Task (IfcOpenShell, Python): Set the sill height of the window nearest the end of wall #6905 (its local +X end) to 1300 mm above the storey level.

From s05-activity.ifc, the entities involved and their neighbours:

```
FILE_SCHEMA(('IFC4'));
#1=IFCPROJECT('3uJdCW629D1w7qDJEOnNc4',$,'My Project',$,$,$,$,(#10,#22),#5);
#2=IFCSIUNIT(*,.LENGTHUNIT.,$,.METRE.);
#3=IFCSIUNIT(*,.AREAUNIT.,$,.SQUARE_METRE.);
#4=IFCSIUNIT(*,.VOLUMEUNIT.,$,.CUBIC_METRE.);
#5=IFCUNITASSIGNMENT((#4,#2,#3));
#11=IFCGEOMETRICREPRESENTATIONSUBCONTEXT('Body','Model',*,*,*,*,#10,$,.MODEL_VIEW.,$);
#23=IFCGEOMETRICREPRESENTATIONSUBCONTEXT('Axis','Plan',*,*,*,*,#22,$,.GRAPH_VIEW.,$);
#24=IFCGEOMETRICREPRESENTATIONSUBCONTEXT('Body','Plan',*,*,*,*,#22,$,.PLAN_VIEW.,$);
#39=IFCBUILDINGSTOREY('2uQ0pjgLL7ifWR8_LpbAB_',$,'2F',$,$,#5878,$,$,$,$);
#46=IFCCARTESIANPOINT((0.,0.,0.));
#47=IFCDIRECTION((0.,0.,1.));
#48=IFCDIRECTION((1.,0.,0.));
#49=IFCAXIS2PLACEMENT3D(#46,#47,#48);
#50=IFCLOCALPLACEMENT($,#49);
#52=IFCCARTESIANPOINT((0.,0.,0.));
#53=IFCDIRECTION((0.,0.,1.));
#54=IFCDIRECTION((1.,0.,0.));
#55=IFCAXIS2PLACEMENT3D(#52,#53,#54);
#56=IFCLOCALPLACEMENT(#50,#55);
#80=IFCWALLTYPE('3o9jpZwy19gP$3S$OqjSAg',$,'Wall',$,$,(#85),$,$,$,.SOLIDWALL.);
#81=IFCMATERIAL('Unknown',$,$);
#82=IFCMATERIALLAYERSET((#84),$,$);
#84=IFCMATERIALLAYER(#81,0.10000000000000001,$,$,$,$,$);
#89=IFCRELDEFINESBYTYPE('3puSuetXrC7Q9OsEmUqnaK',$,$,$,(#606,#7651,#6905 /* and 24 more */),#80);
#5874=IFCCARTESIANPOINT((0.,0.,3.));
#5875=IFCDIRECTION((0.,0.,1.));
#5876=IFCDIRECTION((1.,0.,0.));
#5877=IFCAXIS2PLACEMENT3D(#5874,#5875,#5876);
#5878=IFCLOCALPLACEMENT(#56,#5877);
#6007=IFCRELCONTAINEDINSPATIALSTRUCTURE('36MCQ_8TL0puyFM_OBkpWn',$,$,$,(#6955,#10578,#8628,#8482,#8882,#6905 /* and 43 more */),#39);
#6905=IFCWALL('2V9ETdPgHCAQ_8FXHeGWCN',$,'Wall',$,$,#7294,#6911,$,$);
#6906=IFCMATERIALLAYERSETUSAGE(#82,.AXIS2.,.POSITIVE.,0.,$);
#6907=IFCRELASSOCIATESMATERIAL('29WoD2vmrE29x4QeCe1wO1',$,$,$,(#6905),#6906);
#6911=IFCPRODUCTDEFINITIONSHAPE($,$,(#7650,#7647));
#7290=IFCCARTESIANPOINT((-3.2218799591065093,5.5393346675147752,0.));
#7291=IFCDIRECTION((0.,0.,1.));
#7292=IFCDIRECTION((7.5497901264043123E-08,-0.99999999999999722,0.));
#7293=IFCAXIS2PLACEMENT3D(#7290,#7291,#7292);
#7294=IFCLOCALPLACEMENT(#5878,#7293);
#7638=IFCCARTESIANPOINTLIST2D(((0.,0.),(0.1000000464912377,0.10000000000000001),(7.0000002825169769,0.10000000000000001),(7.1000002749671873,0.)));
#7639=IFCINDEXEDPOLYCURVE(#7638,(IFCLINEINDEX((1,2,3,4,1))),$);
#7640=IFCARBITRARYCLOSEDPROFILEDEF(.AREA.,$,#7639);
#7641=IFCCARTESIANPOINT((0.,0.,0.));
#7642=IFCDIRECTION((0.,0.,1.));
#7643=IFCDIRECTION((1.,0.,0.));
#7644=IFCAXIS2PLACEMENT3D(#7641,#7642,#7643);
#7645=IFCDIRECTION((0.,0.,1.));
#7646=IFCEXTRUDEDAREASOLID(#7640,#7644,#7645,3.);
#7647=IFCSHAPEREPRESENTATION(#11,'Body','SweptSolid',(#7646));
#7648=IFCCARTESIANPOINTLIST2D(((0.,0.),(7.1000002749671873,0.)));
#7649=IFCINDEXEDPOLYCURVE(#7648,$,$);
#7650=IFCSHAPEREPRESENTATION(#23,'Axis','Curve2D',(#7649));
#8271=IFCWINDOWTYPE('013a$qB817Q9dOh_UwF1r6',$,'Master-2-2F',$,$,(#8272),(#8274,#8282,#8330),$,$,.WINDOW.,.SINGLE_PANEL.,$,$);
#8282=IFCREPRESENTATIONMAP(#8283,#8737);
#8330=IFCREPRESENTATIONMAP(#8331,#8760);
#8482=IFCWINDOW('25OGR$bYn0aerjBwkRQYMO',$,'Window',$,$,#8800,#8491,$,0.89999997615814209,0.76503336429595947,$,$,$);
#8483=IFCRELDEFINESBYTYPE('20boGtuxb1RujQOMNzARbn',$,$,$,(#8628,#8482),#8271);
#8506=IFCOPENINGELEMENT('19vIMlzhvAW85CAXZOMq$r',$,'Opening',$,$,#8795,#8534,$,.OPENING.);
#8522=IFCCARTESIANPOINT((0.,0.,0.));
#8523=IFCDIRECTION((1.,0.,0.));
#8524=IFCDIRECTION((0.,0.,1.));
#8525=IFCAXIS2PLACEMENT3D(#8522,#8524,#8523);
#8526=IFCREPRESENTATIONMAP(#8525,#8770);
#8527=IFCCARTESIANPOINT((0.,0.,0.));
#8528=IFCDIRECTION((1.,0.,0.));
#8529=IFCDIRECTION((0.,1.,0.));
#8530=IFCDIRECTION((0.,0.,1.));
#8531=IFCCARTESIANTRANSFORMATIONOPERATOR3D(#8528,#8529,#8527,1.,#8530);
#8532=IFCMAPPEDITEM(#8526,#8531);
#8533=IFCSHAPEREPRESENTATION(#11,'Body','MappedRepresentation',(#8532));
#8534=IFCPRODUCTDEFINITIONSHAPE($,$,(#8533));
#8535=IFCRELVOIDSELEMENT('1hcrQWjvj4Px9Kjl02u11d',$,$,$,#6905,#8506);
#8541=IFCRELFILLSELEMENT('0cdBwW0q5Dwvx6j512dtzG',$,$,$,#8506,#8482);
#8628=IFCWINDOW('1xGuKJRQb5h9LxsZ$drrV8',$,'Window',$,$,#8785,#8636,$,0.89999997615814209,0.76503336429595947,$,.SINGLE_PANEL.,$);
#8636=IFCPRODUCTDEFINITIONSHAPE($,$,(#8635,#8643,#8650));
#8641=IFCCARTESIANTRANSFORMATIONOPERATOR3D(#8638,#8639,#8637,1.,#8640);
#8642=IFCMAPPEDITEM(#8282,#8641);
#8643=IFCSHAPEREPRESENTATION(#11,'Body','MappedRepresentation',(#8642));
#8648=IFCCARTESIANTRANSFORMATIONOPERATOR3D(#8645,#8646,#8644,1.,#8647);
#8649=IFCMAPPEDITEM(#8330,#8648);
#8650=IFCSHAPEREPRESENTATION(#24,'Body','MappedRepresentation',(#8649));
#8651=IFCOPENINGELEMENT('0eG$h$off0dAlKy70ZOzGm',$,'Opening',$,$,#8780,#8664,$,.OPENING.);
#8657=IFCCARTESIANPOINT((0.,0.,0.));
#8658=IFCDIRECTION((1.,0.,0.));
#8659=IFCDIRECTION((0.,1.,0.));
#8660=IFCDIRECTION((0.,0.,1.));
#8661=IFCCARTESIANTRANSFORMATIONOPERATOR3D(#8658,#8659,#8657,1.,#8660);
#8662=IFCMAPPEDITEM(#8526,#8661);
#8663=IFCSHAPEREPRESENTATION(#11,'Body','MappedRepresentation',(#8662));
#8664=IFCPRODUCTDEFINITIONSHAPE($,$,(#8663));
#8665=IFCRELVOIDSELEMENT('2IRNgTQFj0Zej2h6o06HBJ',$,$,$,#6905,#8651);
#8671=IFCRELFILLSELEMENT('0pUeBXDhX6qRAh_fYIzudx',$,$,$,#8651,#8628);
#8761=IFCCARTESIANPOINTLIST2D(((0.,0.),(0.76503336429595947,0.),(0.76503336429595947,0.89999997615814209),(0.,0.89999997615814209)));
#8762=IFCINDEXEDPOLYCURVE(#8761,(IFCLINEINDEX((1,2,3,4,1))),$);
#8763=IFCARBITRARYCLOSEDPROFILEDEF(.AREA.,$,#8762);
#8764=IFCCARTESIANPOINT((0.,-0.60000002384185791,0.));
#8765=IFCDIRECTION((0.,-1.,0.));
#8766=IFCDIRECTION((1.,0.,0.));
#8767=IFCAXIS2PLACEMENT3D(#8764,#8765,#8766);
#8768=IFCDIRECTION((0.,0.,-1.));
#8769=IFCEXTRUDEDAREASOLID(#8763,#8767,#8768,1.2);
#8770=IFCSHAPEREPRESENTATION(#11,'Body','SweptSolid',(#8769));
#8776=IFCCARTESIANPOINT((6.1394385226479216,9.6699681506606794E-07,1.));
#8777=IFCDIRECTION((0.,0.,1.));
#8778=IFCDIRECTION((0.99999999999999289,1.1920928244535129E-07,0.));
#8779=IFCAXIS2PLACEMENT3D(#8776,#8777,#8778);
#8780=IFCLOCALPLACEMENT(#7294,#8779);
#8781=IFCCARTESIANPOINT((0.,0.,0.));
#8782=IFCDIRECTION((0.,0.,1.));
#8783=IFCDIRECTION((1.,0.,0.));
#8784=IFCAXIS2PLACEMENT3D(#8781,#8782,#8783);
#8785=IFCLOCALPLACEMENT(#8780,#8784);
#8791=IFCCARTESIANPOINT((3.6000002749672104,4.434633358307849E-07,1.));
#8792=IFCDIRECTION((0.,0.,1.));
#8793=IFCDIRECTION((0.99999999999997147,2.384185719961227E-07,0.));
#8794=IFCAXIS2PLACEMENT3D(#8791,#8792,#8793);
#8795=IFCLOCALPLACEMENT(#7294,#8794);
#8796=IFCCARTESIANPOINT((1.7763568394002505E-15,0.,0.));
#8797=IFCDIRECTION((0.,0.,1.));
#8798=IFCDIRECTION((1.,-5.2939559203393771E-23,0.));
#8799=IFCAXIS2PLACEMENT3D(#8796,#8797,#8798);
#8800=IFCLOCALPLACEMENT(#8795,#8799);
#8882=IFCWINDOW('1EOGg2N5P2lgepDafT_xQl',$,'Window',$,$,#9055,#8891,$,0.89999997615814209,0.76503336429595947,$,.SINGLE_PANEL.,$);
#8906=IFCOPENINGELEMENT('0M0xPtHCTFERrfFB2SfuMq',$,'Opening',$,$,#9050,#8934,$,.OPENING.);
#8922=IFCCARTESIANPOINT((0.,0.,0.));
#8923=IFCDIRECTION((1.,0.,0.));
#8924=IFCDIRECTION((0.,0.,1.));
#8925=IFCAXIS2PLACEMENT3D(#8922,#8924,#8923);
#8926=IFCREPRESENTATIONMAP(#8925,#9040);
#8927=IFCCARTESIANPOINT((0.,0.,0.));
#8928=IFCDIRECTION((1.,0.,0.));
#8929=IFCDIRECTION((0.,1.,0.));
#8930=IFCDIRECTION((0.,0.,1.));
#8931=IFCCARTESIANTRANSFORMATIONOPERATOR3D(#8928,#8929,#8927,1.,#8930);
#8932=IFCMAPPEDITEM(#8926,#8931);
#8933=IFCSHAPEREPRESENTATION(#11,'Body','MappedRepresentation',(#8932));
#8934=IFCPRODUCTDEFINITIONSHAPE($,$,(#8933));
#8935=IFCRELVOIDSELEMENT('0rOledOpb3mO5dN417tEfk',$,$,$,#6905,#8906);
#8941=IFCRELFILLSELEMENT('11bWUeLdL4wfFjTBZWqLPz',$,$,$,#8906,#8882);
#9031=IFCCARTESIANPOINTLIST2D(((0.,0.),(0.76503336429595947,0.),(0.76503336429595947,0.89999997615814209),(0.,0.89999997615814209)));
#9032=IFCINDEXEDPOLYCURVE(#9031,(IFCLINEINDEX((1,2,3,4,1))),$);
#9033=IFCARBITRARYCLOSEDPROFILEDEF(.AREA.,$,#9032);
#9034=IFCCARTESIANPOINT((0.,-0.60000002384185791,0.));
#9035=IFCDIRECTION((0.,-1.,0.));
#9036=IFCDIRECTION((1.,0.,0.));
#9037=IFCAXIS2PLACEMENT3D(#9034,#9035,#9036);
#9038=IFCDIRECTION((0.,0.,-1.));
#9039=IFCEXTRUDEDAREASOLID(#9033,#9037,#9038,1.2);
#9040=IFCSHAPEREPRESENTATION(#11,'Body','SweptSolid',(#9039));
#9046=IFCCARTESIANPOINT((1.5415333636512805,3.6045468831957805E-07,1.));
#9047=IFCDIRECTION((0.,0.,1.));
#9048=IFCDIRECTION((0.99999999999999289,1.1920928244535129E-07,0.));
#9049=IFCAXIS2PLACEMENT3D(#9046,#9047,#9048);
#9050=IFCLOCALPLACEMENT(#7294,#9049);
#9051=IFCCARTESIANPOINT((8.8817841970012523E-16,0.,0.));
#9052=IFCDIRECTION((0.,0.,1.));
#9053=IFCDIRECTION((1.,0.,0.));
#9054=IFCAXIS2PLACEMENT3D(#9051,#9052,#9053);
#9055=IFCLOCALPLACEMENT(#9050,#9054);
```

```python
import numpy as np
import ifcopenshell
import ifcopenshell.api.geometry
import ifcopenshell.geom
import ifcopenshell.util.element
import ifcopenshell.util.placement
import ifcopenshell.util.shape
import ifcopenshell.util.unit

model = ifcopenshell.open("s05-activity.ifc")
unit_scale = ifcopenshell.util.unit.calculate_unit_scale(model)

window = model.by_guid("1xGuKJRQb5h9LxsZ$drrV8")
opening = window.FillsVoids[0].RelatingOpeningElement
storey = ifcopenshell.util.element.get_container(window, ifc_class="IfcBuildingStorey")
level = ifcopenshell.util.placement.get_local_placement(storey.ObjectPlacement)[2, 3]

# The opening's origin need not be at the sill, so measure its lowest point.
shape = ifcopenshell.geom.create_shape(ifcopenshell.geom.settings(), opening)
bottom = ifcopenshell.util.shape.get_shape_bottom_elevation(shape, shape.geometry) / unit_scale
dz = level + 1.3 - bottom

shift = np.array([0.0, 0.0, dz])
# The window is placed relative to its opening, so it follows when the opening moves.
matrix = ifcopenshell.util.placement.get_local_placement(opening.ObjectPlacement)
matrix[:3, 3] += shift
ifcopenshell.api.geometry.edit_object_placement(
    model, product=opening, matrix=matrix, is_si=False, should_transform_children=True
)

print(f"moved by {dz * unit_scale:+.3f} m")

model.write("s05-activity_v2.ifc")
```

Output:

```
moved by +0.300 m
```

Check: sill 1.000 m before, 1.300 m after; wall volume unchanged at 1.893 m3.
